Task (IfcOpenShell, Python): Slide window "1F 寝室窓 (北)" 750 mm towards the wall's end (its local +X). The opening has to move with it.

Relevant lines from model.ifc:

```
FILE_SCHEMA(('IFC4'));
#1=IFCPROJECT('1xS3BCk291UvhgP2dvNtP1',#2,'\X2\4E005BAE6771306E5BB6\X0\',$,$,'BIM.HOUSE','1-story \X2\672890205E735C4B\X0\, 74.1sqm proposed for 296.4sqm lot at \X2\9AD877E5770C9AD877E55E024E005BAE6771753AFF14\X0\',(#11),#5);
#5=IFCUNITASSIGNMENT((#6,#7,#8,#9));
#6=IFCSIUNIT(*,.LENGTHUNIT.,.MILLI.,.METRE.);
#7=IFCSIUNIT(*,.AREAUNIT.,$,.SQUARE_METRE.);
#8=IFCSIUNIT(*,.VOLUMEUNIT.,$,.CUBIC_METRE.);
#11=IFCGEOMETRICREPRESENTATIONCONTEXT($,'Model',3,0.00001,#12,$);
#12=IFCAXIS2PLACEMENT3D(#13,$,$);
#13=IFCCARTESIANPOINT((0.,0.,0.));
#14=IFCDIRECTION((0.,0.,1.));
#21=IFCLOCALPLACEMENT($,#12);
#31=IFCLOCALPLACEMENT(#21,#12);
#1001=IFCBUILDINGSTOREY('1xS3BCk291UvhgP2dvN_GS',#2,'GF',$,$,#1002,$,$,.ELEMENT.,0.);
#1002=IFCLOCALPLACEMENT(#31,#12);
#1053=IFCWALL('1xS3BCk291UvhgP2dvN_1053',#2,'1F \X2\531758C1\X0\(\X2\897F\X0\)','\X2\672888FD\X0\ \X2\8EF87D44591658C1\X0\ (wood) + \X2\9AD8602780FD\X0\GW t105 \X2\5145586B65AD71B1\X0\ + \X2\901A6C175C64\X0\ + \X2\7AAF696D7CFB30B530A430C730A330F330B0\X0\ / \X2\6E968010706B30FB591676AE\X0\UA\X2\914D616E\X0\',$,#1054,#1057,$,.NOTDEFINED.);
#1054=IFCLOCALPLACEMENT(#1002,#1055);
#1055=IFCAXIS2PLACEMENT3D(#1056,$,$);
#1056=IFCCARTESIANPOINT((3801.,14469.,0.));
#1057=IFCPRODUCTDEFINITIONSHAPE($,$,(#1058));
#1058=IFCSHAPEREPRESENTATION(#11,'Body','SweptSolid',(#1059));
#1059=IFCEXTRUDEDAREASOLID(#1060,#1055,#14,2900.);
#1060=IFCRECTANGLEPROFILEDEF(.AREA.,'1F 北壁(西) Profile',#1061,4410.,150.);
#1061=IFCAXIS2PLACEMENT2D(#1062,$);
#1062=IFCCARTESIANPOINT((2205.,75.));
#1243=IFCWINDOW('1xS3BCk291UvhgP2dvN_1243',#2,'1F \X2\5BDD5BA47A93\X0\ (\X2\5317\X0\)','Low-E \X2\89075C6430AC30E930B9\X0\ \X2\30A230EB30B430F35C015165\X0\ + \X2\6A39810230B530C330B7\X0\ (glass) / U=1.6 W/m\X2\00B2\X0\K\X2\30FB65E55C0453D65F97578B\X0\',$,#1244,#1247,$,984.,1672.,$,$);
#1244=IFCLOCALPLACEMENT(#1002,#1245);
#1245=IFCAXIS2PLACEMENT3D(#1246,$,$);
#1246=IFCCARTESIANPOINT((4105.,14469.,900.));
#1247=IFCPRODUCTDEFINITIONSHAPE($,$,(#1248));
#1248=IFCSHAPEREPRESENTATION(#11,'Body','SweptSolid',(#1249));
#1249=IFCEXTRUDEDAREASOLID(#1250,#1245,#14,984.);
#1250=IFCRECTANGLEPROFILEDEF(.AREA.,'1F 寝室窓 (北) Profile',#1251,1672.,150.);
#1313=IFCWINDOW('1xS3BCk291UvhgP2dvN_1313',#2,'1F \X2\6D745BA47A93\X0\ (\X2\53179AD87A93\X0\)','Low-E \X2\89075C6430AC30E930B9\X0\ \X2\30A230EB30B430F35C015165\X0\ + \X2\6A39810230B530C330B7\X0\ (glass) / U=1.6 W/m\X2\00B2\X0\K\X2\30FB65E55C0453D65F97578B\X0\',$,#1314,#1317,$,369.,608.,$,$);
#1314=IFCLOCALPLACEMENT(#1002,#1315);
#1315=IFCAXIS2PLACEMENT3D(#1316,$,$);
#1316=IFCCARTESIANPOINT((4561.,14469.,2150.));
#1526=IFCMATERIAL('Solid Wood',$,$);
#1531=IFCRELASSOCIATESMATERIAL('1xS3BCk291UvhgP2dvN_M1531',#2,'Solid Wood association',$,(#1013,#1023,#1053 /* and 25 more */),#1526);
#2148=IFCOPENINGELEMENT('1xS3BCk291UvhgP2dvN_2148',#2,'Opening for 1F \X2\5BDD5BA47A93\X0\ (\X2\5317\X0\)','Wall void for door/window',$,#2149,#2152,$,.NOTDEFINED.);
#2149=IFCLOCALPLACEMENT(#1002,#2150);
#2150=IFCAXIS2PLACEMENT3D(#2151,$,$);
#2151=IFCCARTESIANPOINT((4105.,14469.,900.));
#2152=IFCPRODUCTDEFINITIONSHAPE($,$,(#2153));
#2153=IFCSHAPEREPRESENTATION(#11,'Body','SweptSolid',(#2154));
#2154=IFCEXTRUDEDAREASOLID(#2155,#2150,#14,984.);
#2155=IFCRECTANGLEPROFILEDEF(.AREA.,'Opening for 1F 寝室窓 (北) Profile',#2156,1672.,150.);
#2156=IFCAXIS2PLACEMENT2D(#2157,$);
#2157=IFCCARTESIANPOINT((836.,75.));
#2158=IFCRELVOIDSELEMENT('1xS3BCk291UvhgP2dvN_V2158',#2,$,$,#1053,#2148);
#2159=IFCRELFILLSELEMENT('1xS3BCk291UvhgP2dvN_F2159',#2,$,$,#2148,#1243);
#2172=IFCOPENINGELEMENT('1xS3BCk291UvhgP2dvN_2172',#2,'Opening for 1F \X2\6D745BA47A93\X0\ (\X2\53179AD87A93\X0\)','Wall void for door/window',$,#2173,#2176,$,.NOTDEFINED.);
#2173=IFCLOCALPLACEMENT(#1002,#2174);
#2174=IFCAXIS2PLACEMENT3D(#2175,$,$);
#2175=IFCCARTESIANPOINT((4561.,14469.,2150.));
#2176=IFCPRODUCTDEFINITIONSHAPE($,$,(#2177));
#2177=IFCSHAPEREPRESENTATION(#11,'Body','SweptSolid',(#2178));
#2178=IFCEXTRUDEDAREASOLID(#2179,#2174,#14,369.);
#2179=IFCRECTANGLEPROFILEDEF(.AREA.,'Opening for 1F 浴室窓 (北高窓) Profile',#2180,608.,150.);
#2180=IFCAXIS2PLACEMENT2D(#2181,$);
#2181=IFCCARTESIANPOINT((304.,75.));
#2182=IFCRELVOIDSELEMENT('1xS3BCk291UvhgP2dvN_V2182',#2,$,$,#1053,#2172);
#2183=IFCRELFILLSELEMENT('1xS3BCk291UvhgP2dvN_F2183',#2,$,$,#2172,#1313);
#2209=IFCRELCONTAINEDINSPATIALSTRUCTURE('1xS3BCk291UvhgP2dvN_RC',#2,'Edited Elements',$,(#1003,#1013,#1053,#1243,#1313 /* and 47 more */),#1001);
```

```python
import ifcopenshell
import ifcopenshell.api.geometry
import ifcopenshell.util.placement

model = ifcopenshell.open("model.ifc")

window = model.by_guid("1xS3BCk291UvhgP2dvN_1243")
opening = window.FillsVoids[0].RelatingOpeningElement
wall = opening.VoidsElements[0].RelatingBuildingElement

wall_matrix = ifcopenshell.util.placement.get_local_placement(wall.ObjectPlacement)
shift = wall_matrix[:3, 0] * 750.0
before = ifcopenshell.util.placement.get_local_placement(window.ObjectPlacement)[:3, 3].copy()

# The window is not placed relative to its opening, so move both.
for product in (opening, window):
    matrix = ifcopenshell.util.placement.get_local_placement(product.ObjectPlacement)
    matrix[:3, 3] += shift
    ifcopenshell.api.geometry.edit_object_placement(model, product=product, matrix=matrix, is_si=False)

after = ifcopenshell.util.placement.get_local_placement(window.ObjectPlacement)[:3, 3]
print("window moved by", (after - before).round(3) + 0.0)

model.write("model_v2.ifc")
```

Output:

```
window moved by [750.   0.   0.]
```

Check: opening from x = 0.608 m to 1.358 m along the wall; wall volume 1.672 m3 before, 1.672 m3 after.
